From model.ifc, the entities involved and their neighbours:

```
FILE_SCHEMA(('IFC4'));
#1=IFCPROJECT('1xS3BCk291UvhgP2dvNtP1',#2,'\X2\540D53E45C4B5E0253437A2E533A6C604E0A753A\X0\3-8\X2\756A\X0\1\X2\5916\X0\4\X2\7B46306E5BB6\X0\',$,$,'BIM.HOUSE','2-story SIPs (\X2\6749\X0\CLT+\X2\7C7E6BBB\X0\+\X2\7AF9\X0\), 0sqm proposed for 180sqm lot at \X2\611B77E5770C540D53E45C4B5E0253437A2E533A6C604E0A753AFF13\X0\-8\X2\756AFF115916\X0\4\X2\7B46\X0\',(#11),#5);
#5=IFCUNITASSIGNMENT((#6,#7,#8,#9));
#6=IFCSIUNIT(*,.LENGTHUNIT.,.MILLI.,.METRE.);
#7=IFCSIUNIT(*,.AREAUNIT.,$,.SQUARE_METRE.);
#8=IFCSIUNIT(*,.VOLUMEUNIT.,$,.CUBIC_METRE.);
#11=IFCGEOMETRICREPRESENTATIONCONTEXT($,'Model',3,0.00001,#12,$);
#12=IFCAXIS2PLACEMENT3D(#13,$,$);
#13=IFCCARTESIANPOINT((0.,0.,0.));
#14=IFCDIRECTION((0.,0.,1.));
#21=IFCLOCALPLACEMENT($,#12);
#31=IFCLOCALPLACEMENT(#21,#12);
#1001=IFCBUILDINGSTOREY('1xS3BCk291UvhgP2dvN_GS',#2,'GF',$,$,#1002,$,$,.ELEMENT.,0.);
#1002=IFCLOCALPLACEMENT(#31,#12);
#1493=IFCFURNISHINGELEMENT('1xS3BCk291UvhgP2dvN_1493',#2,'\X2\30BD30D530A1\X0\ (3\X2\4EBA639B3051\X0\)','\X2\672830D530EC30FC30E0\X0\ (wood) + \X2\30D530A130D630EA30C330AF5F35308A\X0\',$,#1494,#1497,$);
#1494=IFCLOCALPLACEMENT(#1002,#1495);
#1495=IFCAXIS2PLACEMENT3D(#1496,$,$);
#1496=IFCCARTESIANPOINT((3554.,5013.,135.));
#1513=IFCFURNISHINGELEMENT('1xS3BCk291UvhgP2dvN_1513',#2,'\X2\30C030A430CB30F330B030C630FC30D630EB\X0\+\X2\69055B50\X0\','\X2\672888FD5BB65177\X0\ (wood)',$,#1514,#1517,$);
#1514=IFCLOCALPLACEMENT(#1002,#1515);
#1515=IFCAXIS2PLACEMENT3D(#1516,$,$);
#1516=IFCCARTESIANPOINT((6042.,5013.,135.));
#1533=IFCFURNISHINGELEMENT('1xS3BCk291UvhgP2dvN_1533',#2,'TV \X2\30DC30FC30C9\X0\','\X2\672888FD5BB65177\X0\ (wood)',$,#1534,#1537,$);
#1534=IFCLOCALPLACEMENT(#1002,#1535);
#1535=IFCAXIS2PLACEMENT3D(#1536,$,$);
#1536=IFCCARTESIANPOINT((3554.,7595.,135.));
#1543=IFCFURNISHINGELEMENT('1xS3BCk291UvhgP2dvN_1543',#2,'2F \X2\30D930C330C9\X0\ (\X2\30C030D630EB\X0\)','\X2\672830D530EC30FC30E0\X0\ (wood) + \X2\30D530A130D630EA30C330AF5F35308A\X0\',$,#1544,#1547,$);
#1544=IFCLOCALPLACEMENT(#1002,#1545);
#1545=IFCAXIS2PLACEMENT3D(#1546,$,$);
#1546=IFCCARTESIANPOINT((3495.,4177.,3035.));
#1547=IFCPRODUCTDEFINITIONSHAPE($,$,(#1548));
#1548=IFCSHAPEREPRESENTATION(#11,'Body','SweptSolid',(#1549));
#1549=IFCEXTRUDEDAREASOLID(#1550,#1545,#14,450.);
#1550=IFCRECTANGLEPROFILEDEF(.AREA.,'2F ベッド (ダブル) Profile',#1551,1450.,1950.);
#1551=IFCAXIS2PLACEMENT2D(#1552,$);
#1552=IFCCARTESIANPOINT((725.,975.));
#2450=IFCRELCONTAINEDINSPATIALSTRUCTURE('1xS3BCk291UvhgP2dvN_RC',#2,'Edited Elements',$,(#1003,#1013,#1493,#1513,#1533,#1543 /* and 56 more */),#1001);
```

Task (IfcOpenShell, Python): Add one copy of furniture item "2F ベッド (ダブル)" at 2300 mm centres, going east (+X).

```python
import numpy as np
import ifcopenshell
import ifcopenshell.api.geometry
import ifcopenshell.api.root
import ifcopenshell.util.element
import ifcopenshell.util.placement

model = ifcopenshell.open("model.ifc")


def reuse_history(source, copy):
    """copy_class also copies each property set's owner history, people and application; keep the originals."""
    for rel in copy.IsDefinedBy:
        if rel.is_a("IfcRelDefinesByProperties") and (history := rel.RelatingPropertyDefinition.OwnerHistory):
            rel.RelatingPropertyDefinition.OwnerHistory = source.OwnerHistory
            ifcopenshell.util.element.remove_deep2(model, history)


source = model.by_guid("1xS3BCk291UvhgP2dvN_1543")
base = ifcopenshell.util.placement.get_local_placement(source.ObjectPlacement)
step = np.array([1.0, 0.0, 0.0]) * 2300.0

for i in range(1, 2):
    copy = ifcopenshell.api.root.copy_class(model, product=source)
    copy.Representation = ifcopenshell.util.element.copy_deep(
        model, source.Representation, exclude=["IfcGeometricRepresentationContext", "IfcRepresentationMap"]
    )
    reuse_history(source, copy)
    matrix = base.copy()
    matrix[:3, 3] += i * step
    print("added at", matrix[:3, 3].round(3) + 0.0)
    ifcopenshell.api.geometry.edit_object_placement(model, product=copy, matrix=matrix, is_si=False)

model.write("model_updated.ifc")
```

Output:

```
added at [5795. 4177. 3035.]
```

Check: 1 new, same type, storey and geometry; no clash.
